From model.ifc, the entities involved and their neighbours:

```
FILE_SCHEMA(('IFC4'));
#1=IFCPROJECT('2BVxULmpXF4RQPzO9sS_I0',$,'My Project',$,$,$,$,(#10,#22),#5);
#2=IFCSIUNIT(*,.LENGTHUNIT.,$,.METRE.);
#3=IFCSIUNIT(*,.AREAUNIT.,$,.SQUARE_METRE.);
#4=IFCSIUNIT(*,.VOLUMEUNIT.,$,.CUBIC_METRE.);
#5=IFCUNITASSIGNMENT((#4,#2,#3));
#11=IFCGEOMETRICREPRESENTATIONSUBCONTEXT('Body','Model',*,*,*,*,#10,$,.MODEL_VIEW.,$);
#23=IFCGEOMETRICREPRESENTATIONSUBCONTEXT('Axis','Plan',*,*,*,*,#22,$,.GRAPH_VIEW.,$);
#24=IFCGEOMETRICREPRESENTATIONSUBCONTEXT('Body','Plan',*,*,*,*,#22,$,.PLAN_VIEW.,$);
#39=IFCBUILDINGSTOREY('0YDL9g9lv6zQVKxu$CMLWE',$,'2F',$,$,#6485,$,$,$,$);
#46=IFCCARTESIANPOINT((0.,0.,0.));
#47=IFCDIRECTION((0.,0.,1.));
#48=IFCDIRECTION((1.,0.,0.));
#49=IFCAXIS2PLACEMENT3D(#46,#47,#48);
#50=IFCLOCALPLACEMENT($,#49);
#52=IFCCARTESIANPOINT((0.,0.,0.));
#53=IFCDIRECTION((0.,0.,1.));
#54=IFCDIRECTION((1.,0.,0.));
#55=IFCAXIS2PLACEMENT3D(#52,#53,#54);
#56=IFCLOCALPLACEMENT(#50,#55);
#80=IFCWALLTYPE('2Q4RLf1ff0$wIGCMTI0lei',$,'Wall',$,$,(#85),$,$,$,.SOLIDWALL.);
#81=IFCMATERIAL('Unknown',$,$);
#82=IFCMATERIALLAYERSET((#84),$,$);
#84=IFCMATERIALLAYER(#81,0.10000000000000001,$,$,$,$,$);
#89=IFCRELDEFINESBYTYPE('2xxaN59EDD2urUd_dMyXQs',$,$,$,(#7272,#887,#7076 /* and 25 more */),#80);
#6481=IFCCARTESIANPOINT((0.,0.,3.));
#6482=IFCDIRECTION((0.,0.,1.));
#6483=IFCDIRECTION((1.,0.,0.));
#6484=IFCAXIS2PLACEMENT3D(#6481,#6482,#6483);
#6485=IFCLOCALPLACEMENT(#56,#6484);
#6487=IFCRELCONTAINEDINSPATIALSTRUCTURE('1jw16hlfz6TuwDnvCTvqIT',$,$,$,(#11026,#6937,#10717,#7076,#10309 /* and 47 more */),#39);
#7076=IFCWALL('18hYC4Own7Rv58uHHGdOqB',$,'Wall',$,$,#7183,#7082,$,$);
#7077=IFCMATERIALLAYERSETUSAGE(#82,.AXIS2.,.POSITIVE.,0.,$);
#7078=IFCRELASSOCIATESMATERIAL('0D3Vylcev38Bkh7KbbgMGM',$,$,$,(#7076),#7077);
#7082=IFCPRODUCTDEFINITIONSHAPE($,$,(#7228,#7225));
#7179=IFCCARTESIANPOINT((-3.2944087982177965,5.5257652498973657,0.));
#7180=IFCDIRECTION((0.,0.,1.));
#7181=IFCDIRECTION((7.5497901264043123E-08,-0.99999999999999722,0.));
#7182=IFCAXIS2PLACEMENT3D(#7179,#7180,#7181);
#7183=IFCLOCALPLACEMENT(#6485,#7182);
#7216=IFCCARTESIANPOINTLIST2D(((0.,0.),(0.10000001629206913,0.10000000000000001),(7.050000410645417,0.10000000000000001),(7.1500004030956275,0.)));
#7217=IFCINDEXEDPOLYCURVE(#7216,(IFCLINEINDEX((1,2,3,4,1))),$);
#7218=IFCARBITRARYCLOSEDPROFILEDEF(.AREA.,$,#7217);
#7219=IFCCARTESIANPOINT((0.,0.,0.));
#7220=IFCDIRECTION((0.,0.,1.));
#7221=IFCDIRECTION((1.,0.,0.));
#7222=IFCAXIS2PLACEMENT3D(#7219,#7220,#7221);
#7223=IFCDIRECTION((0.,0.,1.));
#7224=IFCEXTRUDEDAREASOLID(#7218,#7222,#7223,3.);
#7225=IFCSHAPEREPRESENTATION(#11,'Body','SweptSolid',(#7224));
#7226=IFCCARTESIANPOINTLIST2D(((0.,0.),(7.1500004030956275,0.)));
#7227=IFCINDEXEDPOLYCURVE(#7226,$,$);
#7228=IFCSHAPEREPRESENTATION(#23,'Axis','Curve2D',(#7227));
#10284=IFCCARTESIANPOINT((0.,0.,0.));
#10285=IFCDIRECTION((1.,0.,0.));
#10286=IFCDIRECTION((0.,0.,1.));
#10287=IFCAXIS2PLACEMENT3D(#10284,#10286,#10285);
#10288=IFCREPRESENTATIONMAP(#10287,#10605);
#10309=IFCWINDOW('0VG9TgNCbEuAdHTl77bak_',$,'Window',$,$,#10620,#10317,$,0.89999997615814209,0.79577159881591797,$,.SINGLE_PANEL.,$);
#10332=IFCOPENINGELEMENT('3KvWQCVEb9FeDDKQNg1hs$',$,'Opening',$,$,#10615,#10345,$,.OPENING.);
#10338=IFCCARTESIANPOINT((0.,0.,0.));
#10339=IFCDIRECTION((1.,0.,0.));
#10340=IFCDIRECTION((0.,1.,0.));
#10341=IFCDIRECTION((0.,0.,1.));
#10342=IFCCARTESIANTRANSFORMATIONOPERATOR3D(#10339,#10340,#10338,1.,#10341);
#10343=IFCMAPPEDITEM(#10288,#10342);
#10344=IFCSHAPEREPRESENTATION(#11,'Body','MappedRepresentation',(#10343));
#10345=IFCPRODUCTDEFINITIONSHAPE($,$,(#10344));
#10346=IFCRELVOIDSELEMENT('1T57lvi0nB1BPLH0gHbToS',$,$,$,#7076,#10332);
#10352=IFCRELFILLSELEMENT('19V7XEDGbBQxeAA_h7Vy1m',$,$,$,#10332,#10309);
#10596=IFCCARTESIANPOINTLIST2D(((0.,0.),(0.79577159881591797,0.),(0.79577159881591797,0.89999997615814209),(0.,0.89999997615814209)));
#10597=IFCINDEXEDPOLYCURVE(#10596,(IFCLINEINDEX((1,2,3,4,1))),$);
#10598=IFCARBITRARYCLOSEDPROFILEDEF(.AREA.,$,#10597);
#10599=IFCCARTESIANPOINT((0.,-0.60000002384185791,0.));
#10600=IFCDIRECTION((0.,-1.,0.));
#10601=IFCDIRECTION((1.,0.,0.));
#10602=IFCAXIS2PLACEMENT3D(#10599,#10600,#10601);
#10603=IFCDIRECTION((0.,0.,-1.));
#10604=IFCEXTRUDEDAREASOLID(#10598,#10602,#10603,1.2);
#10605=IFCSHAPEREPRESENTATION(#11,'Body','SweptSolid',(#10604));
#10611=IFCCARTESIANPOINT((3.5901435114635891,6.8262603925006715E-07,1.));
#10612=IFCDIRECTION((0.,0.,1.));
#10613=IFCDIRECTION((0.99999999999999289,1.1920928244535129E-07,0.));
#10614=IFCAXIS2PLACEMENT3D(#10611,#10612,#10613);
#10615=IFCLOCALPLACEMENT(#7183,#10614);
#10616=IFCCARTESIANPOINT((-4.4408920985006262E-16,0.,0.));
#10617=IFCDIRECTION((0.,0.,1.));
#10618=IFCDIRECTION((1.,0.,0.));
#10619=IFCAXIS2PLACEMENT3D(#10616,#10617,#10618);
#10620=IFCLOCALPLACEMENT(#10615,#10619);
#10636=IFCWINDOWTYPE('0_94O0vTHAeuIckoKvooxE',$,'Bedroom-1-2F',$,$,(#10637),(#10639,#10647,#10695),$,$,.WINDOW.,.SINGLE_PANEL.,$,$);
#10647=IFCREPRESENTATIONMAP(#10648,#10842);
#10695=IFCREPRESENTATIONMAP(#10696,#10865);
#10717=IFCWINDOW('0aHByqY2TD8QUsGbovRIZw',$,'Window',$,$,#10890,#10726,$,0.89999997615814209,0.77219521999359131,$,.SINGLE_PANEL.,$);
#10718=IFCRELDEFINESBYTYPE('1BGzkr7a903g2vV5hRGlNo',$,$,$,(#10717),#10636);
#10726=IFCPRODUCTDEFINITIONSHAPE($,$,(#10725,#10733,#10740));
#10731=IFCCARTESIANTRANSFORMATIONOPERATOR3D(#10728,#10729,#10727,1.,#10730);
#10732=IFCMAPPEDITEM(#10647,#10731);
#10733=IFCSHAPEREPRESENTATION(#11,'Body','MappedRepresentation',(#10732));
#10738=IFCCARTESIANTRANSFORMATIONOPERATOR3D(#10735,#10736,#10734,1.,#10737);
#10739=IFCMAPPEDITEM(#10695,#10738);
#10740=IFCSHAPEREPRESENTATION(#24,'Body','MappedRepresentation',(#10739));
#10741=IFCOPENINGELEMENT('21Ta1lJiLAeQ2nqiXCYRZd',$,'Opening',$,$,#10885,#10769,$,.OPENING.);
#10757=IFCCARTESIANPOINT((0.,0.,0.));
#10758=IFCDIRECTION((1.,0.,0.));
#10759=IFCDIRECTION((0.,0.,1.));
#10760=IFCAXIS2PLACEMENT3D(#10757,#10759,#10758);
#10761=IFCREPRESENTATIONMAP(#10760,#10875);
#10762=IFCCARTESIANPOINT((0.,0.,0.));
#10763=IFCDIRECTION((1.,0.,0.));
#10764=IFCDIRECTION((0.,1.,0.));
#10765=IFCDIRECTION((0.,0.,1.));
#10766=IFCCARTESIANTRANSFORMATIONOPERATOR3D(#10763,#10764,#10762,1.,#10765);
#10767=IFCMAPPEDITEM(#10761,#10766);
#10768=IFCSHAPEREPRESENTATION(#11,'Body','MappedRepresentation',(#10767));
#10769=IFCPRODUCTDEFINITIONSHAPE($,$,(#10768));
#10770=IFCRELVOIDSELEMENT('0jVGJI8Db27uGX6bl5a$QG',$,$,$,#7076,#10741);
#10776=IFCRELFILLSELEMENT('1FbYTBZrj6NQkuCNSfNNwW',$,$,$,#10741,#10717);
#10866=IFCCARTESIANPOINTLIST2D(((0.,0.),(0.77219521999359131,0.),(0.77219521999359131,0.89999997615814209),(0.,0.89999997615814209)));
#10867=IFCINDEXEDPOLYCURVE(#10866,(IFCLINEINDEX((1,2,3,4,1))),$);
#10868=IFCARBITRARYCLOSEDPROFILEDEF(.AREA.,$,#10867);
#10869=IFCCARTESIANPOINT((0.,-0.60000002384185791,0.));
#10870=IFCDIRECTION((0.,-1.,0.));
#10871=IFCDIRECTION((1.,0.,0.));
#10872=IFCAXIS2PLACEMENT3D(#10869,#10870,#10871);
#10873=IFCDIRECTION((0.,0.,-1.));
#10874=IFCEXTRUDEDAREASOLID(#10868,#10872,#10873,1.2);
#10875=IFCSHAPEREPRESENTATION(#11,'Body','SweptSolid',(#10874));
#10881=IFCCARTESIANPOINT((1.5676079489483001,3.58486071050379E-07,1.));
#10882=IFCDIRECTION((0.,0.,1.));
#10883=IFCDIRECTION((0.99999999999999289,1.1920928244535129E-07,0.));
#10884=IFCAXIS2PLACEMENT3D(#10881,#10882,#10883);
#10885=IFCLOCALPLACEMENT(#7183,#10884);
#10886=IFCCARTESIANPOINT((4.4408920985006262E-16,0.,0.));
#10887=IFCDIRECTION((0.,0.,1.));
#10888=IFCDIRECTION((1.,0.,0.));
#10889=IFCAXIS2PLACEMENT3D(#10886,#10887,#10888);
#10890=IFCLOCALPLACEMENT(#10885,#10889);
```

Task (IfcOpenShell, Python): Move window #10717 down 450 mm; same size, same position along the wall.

```python
import numpy as np
import ifcopenshell
import ifcopenshell.api.geometry
import ifcopenshell.util.placement
import ifcopenshell.util.unit

model = ifcopenshell.open("model.ifc")
unit_scale = ifcopenshell.util.unit.calculate_unit_scale(model)

window = model.by_guid("0aHByqY2TD8QUsGbovRIZw")
opening = window.FillsVoids[0].RelatingOpeningElement
dz = -0.45

shift = np.array([0.0, 0.0, dz])
# The window is placed relative to its opening, so it follows when the opening moves.
matrix = ifcopenshell.util.placement.get_local_placement(opening.ObjectPlacement)
matrix[:3, 3] += shift
ifcopenshell.api.geometry.edit_object_placement(
    model, product=opening, matrix=matrix, is_si=False, should_transform_children=True
)

print(f"moved by {dz * unit_scale:+.3f} m")

model.write("model_rev.ifc")
```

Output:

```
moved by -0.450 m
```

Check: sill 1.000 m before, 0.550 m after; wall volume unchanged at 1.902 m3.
